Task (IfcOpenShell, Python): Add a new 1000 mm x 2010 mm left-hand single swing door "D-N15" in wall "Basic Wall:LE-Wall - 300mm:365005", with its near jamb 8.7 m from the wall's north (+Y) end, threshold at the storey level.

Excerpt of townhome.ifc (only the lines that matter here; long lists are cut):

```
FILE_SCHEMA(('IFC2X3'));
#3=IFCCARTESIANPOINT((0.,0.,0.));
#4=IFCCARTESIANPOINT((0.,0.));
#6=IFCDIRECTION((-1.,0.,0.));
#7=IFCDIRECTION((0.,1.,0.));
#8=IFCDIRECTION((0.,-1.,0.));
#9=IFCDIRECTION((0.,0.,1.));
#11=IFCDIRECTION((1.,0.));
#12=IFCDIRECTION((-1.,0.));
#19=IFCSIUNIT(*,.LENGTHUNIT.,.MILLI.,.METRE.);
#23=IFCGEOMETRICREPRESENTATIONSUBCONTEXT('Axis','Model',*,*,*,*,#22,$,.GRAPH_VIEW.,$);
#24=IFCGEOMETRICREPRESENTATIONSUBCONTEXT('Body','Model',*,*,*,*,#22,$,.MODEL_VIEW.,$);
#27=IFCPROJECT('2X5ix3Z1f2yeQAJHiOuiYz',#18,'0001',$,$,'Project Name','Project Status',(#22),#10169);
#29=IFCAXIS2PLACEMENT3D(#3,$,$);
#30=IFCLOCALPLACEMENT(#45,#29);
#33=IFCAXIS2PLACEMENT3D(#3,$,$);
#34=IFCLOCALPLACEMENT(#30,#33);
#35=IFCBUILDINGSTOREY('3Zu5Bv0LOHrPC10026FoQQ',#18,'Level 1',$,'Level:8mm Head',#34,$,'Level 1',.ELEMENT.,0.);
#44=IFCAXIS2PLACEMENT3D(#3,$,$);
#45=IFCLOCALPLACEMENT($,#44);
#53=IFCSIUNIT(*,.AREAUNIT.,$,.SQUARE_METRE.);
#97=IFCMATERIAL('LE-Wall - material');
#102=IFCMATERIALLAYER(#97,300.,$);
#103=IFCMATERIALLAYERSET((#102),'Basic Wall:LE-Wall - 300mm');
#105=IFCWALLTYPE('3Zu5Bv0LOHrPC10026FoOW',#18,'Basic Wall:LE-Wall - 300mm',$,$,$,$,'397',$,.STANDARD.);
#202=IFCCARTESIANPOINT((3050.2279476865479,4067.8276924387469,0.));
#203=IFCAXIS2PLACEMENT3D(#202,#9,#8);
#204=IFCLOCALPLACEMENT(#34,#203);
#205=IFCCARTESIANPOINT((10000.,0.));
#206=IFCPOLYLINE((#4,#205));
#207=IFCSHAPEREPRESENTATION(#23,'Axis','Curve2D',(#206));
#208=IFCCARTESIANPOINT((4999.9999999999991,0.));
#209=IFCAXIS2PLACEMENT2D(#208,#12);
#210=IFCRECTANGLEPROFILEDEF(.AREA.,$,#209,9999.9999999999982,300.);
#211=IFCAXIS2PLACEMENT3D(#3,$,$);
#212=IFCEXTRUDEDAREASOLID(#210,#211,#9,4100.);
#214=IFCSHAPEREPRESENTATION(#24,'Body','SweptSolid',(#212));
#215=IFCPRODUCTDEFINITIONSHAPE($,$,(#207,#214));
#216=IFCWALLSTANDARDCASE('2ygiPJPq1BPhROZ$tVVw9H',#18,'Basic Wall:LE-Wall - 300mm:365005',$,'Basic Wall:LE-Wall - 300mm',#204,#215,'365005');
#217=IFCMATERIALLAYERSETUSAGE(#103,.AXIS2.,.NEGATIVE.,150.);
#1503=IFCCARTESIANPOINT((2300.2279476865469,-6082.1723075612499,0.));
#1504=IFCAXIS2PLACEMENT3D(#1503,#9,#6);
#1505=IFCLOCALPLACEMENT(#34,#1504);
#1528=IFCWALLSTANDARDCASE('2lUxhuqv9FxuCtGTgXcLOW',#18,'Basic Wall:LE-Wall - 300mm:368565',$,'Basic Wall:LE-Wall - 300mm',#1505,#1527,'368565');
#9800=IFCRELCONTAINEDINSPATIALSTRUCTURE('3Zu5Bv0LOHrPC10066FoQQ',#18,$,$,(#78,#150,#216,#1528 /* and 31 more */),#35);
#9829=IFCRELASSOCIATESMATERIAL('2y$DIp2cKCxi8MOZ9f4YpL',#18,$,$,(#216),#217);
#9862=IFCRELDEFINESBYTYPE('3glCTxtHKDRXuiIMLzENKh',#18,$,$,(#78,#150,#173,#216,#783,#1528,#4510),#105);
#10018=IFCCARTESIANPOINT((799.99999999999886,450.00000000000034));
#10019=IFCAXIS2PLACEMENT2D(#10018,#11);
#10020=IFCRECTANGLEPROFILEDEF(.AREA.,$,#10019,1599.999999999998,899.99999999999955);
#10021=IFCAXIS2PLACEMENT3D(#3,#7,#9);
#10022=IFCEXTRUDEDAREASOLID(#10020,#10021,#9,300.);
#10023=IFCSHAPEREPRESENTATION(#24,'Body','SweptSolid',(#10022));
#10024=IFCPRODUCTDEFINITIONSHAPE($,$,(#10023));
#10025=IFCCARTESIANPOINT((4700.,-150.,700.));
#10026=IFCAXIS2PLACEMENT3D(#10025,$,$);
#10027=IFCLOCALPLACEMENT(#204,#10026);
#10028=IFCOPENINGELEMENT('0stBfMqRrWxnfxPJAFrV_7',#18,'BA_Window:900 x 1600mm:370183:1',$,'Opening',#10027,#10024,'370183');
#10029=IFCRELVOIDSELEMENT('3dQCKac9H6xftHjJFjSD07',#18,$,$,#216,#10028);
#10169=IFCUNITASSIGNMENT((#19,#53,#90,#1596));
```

```python
import numpy as np
import ifcopenshell
import ifcopenshell.api.feature
import ifcopenshell.api.geometry
import ifcopenshell.api.root
import ifcopenshell.api.spatial
import ifcopenshell.api.type
import ifcopenshell.geom
import ifcopenshell.util.element
import ifcopenshell.util.placement
import ifcopenshell.util.representation
import ifcopenshell.util.shape
import ifcopenshell.util.unit

model = ifcopenshell.open("townhome.ifc")
unit_scale = ifcopenshell.util.unit.calculate_unit_scale(model)
settings = ifcopenshell.geom.settings()


def volume(element):
    """Net volume in cubic metres, openings subtracted."""
    shape = ifcopenshell.geom.create_shape(settings, element)
    return ifcopenshell.util.shape.get_volume(shape.geometry)


wall = model.by_guid("2ygiPJPq1BPhROZ$tVVw9H")
storey = ifcopenshell.util.element.get_container(wall, ifc_class="IfcBuildingStorey")
context = ifcopenshell.util.representation.get_context(model, "Model", "Body", "MODEL_VIEW")
before = volume(wall)

width, height, from_end, sill = 1, 2.01, 8.7, 0.0  # metres

# The wall runs along its own X axis, and the end named is its -X end.
wall_shape = ifcopenshell.geom.create_shape(settings, wall)
x, y, z = ifcopenshell.util.shape.get_vertices(wall_shape.geometry).T
start = x.min() + from_end
face, thickness = float(y.min()), float(y.max() - y.min())
wall_matrix = ifcopenshell.util.placement.get_local_placement(wall.ObjectPlacement)
level = ifcopenshell.util.placement.get_local_placement(storey.ObjectPlacement)[2, 3]


def in_wall(x, y):
    """Placement at x, y metres in the wall's axes, at sill height."""
    matrix = wall_matrix.copy()
    matrix[:, 3] = wall_matrix @ np.array([x / unit_scale, y / unit_scale, 0.0, 1.0])
    matrix[2, 3] = level + sill / unit_scale
    return matrix


# Opening: a box that overshoots both wall faces by 50 mm.
opening = ifcopenshell.api.root.create_entity(model, ifc_class="IfcOpeningElement")
box = ifcopenshell.api.geometry.add_wall_representation(
    model, context=context, length=width, height=height, thickness=thickness + 0.1
)
ifcopenshell.api.geometry.assign_representation(model, product=opening, representation=box)
ifcopenshell.api.geometry.edit_object_placement(model, product=opening, matrix=in_wall(start, face - 0.05), is_si=False)
ifcopenshell.api.feature.add_feature(model, feature=opening, element=wall)

door = ifcopenshell.api.root.create_entity(model, ifc_class="IfcDoor", name="D-N15")
door.OverallWidth, door.OverallHeight = width / unit_scale, height / unit_scale
body = ifcopenshell.api.geometry.add_door_representation(
    model,
    context=context,
    overall_width=door.OverallWidth,
    overall_height=door.OverallHeight,
    operation_type="SINGLE_SWING_LEFT",
    lining_properties={"LiningDepth": thickness / unit_scale, "ThresholdDepth": thickness / unit_scale},
)
ifcopenshell.api.geometry.assign_representation(model, product=door, representation=body)
ifcopenshell.api.spatial.assign_container(model, products=[door], relating_structure=storey)
fills = ifcopenshell.api.feature.add_filling(model, opening=opening, element=door)
fills.OwnerHistory = door.OwnerHistory  # required in IFC2X3

# IFC2X3 keeps the operation on the door style.
style = ifcopenshell.api.root.create_entity(model, ifc_class="IfcDoorStyle", name="D-N15")
style.OperationType, style.ConstructionType = "SINGLE_SWING_LEFT", "NOTDEFINED"
style.ParameterTakesPrecedence = style.Sizeable = False
ifcopenshell.api.type.assign_type(model, related_objects=[door], relating_type=style)

# The lining spans the wall, so the door starts at the wall face.
ifcopenshell.api.geometry.edit_object_placement(model, product=door, matrix=in_wall(start, face), is_si=False)

after = volume(wall)

print(f"wall volume {before:.3f} -> {after:.3f} m3")

model.write("townhome_v2.ifc")
```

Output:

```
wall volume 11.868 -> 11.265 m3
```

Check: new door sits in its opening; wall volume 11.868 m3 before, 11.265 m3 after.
